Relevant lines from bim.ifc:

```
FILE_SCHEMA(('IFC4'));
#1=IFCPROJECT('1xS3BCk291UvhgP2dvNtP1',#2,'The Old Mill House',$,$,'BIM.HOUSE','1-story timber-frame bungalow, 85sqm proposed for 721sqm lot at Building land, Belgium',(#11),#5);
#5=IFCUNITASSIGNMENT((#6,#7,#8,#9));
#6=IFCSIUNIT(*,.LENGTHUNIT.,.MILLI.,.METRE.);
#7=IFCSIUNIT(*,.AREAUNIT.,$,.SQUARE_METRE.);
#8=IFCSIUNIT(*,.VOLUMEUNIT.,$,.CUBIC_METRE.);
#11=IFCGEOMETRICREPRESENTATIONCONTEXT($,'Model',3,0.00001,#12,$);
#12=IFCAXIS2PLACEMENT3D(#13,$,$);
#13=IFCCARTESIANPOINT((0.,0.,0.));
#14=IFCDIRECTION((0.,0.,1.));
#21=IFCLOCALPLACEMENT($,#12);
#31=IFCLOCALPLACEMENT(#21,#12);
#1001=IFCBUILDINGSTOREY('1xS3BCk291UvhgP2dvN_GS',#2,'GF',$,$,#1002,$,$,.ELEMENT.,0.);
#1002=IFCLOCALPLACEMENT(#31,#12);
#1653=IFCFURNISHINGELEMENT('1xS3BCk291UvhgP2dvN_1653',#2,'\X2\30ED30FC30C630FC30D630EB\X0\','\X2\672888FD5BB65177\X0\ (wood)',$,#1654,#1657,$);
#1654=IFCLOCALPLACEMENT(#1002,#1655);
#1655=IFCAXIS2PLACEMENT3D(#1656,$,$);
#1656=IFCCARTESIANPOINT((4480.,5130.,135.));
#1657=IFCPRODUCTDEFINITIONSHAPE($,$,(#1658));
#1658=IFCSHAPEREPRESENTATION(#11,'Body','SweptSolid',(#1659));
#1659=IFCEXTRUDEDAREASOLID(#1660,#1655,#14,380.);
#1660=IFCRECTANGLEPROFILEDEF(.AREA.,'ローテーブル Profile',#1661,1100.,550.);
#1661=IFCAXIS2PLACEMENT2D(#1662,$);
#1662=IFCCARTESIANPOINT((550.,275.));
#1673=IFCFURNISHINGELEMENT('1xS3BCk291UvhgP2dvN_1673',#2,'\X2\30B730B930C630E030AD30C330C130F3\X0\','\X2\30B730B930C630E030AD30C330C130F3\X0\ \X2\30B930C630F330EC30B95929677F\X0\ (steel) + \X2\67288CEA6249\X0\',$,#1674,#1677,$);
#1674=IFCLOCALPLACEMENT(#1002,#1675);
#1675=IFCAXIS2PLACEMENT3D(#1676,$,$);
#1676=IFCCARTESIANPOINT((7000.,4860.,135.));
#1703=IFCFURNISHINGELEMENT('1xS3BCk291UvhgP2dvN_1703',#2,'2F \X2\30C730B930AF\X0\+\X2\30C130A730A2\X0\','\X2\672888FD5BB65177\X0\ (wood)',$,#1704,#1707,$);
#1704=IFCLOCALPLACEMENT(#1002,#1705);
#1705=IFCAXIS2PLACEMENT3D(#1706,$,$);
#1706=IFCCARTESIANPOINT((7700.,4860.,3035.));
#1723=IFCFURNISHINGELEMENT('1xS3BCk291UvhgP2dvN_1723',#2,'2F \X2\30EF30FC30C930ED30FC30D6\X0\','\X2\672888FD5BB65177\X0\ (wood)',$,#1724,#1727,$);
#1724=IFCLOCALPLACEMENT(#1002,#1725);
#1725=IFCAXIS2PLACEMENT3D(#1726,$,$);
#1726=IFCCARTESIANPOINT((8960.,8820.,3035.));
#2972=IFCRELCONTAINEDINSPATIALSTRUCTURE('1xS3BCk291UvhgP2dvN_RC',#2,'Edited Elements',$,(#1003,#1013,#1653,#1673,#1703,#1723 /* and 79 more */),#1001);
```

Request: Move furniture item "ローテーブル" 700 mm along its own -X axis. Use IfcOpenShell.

```python
import ifcopenshell
import ifcopenshell.api.geometry
import ifcopenshell.util.placement

model = ifcopenshell.open("bim.ifc")

item = model.by_guid("1xS3BCk291UvhgP2dvN_1653")
matrix = ifcopenshell.util.placement.get_local_placement(item.ObjectPlacement)
matrix[:3, 3] -= matrix[:3, 0] * 700.0
ifcopenshell.api.geometry.edit_object_placement(model, product=item, matrix=matrix, is_si=False)

print(ifcopenshell.util.placement.get_local_placement(item.ObjectPlacement).round(3) + 0.0)

model.write("bim_rev.ifc")
```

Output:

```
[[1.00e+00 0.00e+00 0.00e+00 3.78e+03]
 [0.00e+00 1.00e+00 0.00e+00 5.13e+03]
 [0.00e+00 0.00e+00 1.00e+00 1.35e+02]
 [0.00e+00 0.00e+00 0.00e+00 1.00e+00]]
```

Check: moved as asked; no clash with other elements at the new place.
